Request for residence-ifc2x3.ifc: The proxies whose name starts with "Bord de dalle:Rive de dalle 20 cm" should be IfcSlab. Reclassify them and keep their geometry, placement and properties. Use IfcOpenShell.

First a look at what the model holds.

```python
import re

import ifcopenshell

model = ifcopenshell.open("residence-ifc2x3.ifc")
print(model.schema)
seen = {}
for e in model.by_type("IfcBuildingElementProxy"):
    name = re.sub(r":\d+(:\d+)?$", "", e.Name or "")  # drop the element id that some exporters append
    seen[name] = seen.get(name, 0) + 1
for name, count in sorted(seen.items()):
    print(count, "x", name)
```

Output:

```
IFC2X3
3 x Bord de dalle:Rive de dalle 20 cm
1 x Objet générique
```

```python
import ifcopenshell
import ifcopenshell.api.root

model = ifcopenshell.open("residence-ifc2x3.ifc")

proxies = [e.id() for e in model.by_type("IfcBuildingElementProxy") if (e.Name or "").startswith("Bord de dalle:Rive de dalle 20 cm")]
for step_id in proxies:
    proxy = model.by_id(step_id)
    # Reclassifying a typed element also reclassifies its type and the type's other occurrences.
    if proxy.is_a("IfcBuildingElementProxy"):
        ifcopenshell.api.root.reassign_class(model, product=proxy, ifc_class="IfcSlab", predefined_type="FLOOR")

print(sum(model.by_id(i).is_a("IfcSlab") for i in proxies), "reclassified")

model.write("residence-ifc2x3_v2.ifc")
```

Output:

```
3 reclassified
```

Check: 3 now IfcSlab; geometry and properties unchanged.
